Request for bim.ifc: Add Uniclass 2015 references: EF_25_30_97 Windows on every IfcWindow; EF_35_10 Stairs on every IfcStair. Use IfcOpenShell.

First a look at what the model holds.

```python
import ifcopenshell

model = ifcopenshell.open("bim.ifc")
print(model.schema)
print("classifications:", [c.Name for c in model.by_type("IfcClassification")])
for ifc_class in ("IfcDoor", "IfcRoof", "IfcStair", "IfcWall", "IfcWindow"):
    print(ifc_class, len(model.by_type(ifc_class)))
```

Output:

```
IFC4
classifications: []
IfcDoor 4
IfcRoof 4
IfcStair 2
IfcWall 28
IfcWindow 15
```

```python
import ifcopenshell
import ifcopenshell.api.classification

model = ifcopenshell.open("bim.ifc")

system = ifcopenshell.api.classification.add_classification(model, classification="Uniclass 2015")

codes = {
    "IfcWindow": ("EF_25_30_97", "Windows"),
    "IfcStair": ("EF_35_10", "Stairs"),
}
for ifc_class, (code, name) in codes.items():
    products = model.by_type(ifc_class)
    ifcopenshell.api.classification.add_reference(
        model, products=products, classification=system, identification=code, name=name
    )
    print(code, len(products))

model.write("bim_v2.ifc")
```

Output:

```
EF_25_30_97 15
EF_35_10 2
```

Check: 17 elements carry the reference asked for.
